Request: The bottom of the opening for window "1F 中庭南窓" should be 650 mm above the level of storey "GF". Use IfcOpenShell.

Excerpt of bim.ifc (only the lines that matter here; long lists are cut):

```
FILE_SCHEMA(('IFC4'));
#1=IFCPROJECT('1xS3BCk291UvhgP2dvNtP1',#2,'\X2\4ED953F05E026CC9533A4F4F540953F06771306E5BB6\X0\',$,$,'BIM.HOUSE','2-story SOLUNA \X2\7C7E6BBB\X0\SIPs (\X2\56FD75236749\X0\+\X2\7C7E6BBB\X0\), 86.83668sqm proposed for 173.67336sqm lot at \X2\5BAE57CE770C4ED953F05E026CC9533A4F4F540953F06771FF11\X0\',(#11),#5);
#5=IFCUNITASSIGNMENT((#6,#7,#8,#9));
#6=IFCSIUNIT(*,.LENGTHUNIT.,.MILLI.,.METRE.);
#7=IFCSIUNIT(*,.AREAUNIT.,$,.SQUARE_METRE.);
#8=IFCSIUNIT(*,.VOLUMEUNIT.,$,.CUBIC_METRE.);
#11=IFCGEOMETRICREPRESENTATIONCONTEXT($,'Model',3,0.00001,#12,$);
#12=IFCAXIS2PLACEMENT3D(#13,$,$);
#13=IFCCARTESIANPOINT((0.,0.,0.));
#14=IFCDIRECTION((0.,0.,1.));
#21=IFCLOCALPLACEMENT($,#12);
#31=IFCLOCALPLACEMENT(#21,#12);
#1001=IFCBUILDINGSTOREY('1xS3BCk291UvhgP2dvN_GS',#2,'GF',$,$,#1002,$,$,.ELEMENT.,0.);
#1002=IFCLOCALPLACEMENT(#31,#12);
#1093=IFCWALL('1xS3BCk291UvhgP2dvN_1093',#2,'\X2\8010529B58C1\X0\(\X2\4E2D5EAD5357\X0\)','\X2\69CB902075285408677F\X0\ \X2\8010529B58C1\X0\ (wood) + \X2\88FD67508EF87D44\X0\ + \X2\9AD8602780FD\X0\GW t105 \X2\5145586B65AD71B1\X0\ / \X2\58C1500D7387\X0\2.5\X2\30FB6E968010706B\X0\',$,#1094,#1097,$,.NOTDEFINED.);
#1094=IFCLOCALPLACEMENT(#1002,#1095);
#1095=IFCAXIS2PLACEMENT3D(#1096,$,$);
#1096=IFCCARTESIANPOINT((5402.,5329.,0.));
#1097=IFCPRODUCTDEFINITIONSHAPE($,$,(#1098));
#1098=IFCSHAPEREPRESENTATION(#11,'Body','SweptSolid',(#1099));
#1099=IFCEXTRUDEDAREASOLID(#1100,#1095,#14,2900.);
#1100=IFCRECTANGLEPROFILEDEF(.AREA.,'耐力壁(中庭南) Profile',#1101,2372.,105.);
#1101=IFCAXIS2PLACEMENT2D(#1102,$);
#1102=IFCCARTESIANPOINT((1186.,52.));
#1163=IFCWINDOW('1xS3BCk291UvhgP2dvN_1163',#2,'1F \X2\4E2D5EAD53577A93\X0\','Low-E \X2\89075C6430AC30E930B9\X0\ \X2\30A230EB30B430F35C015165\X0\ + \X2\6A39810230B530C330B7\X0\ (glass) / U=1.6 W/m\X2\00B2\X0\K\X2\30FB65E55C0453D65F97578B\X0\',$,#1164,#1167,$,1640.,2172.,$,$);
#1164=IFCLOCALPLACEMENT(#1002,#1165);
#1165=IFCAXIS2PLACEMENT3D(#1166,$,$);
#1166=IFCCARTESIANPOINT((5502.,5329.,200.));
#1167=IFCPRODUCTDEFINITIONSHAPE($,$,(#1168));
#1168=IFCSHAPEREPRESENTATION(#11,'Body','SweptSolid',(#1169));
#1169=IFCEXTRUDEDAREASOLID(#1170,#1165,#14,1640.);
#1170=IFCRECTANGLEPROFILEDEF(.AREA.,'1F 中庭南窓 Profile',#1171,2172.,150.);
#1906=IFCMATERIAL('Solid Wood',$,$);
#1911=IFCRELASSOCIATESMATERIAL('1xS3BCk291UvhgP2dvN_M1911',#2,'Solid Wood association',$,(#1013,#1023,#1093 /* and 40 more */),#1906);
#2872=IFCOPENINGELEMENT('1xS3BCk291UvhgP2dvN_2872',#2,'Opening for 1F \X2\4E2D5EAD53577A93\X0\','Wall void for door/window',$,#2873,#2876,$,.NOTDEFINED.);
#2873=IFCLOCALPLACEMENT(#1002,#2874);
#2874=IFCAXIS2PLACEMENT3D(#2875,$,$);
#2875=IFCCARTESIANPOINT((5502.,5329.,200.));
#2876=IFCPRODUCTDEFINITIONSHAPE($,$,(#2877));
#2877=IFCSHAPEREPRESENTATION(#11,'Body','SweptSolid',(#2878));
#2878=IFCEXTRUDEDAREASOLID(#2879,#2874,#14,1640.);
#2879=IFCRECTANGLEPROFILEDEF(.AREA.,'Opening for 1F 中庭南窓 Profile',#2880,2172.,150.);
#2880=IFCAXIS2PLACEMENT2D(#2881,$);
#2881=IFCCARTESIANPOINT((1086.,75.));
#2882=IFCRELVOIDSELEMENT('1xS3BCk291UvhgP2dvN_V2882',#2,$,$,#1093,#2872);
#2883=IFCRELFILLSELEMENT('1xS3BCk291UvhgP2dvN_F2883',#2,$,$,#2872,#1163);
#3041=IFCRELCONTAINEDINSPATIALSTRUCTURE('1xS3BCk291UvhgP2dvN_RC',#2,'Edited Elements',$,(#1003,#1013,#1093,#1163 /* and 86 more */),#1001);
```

```python
import numpy as np
import ifcopenshell
import ifcopenshell.api.geometry
import ifcopenshell.geom
import ifcopenshell.util.element
import ifcopenshell.util.placement
import ifcopenshell.util.shape
import ifcopenshell.util.unit

model = ifcopenshell.open("bim.ifc")
unit_scale = ifcopenshell.util.unit.calculate_unit_scale(model)

window = model.by_id(1163)
opening = window.FillsVoids[0].RelatingOpeningElement
storey = ifcopenshell.util.element.get_container(window, ifc_class="IfcBuildingStorey")
level = ifcopenshell.util.placement.get_local_placement(storey.ObjectPlacement)[2, 3]

# The opening's origin need not be at the sill, so measure its lowest point.
shape = ifcopenshell.geom.create_shape(ifcopenshell.geom.settings(), opening)
bottom = ifcopenshell.util.shape.get_shape_bottom_elevation(shape, shape.geometry) / unit_scale
dz = level + 650.0 - bottom

shift = np.array([0.0, 0.0, dz])
# The window is not placed relative to its opening, so move both.
for product in (opening, window):
    matrix = ifcopenshell.util.placement.get_local_placement(product.ObjectPlacement)
    matrix[:3, 3] += shift
    ifcopenshell.api.geometry.edit_object_placement(model, product=product, matrix=matrix, is_si=False)

print(f"moved by {dz * unit_scale:+.3f} m")

model.write("bim_updated.ifc")
```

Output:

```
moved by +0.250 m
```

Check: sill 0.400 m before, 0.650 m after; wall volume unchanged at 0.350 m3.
